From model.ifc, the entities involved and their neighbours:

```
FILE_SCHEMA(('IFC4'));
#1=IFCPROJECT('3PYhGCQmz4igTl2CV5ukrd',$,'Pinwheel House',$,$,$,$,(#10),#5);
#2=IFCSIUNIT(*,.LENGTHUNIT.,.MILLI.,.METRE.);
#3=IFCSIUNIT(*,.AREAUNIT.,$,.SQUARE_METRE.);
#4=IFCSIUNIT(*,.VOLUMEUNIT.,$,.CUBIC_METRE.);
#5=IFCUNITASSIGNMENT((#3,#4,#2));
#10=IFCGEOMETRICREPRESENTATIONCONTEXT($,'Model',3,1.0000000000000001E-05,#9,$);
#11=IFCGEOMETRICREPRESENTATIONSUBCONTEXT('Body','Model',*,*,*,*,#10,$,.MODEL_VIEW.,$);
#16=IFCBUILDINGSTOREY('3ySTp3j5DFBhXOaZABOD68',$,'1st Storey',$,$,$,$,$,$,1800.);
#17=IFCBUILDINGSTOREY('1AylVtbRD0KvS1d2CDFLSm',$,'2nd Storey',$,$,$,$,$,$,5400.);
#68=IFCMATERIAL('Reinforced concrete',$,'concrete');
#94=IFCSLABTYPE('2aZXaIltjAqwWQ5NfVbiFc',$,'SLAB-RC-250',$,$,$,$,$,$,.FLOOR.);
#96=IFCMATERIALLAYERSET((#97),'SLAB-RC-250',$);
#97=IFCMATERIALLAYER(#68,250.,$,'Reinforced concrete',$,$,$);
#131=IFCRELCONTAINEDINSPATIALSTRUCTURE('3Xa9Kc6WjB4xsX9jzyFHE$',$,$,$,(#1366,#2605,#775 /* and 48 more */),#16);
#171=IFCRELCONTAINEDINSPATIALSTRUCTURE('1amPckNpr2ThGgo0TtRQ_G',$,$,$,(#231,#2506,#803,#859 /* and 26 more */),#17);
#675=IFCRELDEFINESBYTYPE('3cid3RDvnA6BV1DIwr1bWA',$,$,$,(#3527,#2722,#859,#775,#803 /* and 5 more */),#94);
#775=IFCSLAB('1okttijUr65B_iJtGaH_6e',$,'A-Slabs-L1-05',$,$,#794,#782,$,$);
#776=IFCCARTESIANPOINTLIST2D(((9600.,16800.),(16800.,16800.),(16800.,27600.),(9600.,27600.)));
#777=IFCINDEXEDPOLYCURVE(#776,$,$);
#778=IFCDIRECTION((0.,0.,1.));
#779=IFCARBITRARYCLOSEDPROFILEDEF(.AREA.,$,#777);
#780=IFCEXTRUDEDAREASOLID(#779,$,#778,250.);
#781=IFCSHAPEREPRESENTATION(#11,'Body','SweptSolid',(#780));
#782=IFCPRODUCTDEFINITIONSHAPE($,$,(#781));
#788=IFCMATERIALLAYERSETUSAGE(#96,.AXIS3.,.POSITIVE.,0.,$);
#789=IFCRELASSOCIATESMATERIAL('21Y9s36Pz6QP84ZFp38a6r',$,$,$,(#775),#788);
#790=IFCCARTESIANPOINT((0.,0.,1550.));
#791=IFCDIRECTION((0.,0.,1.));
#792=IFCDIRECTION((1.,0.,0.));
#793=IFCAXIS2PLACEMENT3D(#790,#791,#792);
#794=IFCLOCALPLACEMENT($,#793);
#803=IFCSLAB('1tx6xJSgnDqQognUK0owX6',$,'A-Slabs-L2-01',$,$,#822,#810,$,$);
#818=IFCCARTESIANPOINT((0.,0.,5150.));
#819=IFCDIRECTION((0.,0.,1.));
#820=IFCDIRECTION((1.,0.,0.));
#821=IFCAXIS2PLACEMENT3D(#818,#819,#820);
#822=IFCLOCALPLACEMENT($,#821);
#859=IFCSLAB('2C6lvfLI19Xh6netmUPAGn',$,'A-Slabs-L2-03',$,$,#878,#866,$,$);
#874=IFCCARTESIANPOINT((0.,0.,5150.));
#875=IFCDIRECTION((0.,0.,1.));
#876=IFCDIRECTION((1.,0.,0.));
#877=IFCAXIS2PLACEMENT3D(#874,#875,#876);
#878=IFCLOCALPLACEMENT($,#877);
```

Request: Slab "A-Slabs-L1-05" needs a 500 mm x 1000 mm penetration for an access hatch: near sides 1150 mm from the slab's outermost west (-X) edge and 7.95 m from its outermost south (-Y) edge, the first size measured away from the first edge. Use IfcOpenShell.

```python
import numpy as np
import ifcopenshell
import ifcopenshell.api.feature
import ifcopenshell.api.geometry
import ifcopenshell.api.root
import ifcopenshell.geom
import ifcopenshell.util.placement
import ifcopenshell.util.representation
import ifcopenshell.util.shape
import ifcopenshell.util.unit

model = ifcopenshell.open("model.ifc")
unit_scale = ifcopenshell.util.unit.calculate_unit_scale(model)
settings = ifcopenshell.geom.settings()


def volume(element):
    """Net volume in cubic metres, openings subtracted."""
    shape = ifcopenshell.geom.create_shape(settings, element)
    return ifcopenshell.util.shape.get_volume(shape.geometry)


slab = model.by_guid("1okttijUr65B_iJtGaH_6e")
before = volume(slab)

# Extent in the slab's own axes, in metres. The edges named are its -X and -Y sides.
slab_shape = ifcopenshell.geom.create_shape(settings, slab)
vertices = ifcopenshell.util.shape.get_vertices(slab_shape.geometry)
x_min, y_min, bottom = vertices.min(axis=0)
top = vertices[:, 2].max()

opening = ifcopenshell.api.root.create_entity(model, ifc_class="IfcOpeningElement", name="Access hatch opening", predefined_type="OPENING")
context = ifcopenshell.util.representation.get_context(model, "Model", "Body", "MODEL_VIEW")
width, depth = 0.5, 1
outline = [(0.0, 0.0), (width, 0.0), (width, depth), (0.0, depth), (0.0, 0.0)]
# Overshoot both faces by 50 mm so the cut is clean.
shape = ifcopenshell.api.geometry.add_slab_representation(
    model, context=context, depth=top - bottom + 0.1, polyline=outline
)
ifcopenshell.api.geometry.assign_representation(model, product=opening, representation=shape)

matrix = ifcopenshell.util.placement.get_local_placement(slab.ObjectPlacement)
matrix[:, 3] = matrix @ np.append(np.array([x_min + 1.15, y_min + 7.95, bottom - 0.05]) / unit_scale, 1.0)
ifcopenshell.api.geometry.edit_object_placement(model, product=opening, matrix=matrix, is_si=False)
ifcopenshell.api.feature.add_feature(model, feature=opening, element=slab)

after = volume(slab)

print(f"slab volume {before:.3f} -> {after:.3f} m3")

model.write("model_rev.ifc")
```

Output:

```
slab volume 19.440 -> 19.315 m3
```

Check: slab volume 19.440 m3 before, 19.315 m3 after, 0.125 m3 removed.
